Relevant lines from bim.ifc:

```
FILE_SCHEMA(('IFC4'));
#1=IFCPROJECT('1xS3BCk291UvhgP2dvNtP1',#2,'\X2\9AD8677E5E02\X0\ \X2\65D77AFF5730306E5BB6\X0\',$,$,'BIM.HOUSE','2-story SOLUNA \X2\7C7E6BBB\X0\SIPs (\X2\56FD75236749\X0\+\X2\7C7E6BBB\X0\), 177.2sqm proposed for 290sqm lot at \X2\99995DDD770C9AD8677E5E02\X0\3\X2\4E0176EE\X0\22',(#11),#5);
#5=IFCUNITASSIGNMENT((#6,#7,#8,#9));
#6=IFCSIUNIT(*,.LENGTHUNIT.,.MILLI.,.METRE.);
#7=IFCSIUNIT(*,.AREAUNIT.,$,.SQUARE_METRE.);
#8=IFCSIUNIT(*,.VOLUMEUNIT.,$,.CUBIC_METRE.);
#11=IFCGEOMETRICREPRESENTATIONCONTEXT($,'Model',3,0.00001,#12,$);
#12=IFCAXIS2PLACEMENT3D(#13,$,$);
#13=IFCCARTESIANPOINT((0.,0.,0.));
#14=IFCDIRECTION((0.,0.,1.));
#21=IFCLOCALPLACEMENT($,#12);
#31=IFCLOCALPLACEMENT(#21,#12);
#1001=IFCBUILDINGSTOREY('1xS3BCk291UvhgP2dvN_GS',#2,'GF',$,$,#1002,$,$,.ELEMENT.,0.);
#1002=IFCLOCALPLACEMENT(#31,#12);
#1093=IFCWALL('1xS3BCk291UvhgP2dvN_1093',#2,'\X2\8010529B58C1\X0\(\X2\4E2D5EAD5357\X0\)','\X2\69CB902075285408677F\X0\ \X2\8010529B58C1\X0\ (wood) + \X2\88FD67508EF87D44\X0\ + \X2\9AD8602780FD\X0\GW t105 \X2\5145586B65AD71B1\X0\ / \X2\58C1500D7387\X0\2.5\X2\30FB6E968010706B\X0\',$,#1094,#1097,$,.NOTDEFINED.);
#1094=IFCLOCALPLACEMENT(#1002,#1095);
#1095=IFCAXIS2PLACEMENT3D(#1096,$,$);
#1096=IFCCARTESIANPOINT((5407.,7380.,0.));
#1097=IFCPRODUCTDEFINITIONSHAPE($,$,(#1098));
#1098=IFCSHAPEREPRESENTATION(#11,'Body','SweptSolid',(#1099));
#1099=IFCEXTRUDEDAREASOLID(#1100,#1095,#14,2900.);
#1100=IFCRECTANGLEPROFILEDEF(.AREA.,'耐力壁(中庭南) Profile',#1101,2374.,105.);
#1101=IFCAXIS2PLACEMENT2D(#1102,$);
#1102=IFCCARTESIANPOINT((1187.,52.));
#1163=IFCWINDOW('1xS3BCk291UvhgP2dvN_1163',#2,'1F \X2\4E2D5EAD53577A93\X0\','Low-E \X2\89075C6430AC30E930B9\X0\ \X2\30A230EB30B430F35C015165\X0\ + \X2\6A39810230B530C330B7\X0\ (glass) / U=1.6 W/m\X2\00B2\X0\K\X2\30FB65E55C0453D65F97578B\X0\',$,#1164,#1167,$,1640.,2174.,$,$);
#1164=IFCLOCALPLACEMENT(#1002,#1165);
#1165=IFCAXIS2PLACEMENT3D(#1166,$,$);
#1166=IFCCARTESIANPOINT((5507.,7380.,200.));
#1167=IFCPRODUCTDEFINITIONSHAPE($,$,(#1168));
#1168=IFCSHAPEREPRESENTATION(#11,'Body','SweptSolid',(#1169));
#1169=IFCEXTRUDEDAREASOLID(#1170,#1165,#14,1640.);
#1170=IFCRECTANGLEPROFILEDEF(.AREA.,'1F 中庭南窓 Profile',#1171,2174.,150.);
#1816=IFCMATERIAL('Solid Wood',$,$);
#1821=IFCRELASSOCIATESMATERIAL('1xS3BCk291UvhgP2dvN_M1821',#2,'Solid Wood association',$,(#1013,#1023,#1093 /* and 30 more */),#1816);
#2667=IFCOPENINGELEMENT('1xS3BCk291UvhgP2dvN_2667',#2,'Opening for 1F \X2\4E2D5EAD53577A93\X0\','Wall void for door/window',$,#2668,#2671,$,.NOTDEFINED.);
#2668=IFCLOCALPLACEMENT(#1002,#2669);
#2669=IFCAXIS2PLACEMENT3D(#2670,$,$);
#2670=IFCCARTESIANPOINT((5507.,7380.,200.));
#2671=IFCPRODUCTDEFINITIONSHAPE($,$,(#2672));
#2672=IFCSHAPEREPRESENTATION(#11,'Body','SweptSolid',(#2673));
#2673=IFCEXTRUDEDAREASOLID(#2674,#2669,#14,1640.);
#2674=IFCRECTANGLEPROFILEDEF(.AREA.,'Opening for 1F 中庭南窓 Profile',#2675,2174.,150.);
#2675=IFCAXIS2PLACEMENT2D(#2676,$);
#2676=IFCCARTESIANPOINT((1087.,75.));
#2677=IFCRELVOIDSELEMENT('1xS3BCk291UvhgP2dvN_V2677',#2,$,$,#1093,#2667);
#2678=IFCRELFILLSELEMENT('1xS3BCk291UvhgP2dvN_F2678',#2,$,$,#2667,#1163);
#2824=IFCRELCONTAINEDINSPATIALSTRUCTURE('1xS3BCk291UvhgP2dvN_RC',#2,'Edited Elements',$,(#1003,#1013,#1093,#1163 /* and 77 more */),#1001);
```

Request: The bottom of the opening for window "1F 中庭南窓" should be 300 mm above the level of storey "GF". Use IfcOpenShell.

```python
import numpy as np
import ifcopenshell
import ifcopenshell.api.geometry
import ifcopenshell.geom
import ifcopenshell.util.element
import ifcopenshell.util.placement
import ifcopenshell.util.shape
import ifcopenshell.util.unit

model = ifcopenshell.open("bim.ifc")
unit_scale = ifcopenshell.util.unit.calculate_unit_scale(model)

window = model.by_guid("1xS3BCk291UvhgP2dvN_1163")
opening = window.FillsVoids[0].RelatingOpeningElement
storey = ifcopenshell.util.element.get_container(window, ifc_class="IfcBuildingStorey")
level = ifcopenshell.util.placement.get_local_placement(storey.ObjectPlacement)[2, 3]

# The opening's origin need not be at the sill, so measure its lowest point.
shape = ifcopenshell.geom.create_shape(ifcopenshell.geom.settings(), opening)
bottom = ifcopenshell.util.shape.get_shape_bottom_elevation(shape, shape.geometry) / unit_scale
dz = level + 0.3 / unit_scale - bottom

shift = np.array([0.0, 0.0, dz])
# The window is not placed relative to its opening, so move both.
for product in (opening, window):
    matrix = ifcopenshell.util.placement.get_local_placement(product.ObjectPlacement)
    matrix[:3, 3] += shift
    ifcopenshell.api.geometry.edit_object_placement(model, product=product, matrix=matrix, is_si=False)

print(f"moved by {dz * unit_scale:+.3f} m")

model.write("bim_rev.ifc")
```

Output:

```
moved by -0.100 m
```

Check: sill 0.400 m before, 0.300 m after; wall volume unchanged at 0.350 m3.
